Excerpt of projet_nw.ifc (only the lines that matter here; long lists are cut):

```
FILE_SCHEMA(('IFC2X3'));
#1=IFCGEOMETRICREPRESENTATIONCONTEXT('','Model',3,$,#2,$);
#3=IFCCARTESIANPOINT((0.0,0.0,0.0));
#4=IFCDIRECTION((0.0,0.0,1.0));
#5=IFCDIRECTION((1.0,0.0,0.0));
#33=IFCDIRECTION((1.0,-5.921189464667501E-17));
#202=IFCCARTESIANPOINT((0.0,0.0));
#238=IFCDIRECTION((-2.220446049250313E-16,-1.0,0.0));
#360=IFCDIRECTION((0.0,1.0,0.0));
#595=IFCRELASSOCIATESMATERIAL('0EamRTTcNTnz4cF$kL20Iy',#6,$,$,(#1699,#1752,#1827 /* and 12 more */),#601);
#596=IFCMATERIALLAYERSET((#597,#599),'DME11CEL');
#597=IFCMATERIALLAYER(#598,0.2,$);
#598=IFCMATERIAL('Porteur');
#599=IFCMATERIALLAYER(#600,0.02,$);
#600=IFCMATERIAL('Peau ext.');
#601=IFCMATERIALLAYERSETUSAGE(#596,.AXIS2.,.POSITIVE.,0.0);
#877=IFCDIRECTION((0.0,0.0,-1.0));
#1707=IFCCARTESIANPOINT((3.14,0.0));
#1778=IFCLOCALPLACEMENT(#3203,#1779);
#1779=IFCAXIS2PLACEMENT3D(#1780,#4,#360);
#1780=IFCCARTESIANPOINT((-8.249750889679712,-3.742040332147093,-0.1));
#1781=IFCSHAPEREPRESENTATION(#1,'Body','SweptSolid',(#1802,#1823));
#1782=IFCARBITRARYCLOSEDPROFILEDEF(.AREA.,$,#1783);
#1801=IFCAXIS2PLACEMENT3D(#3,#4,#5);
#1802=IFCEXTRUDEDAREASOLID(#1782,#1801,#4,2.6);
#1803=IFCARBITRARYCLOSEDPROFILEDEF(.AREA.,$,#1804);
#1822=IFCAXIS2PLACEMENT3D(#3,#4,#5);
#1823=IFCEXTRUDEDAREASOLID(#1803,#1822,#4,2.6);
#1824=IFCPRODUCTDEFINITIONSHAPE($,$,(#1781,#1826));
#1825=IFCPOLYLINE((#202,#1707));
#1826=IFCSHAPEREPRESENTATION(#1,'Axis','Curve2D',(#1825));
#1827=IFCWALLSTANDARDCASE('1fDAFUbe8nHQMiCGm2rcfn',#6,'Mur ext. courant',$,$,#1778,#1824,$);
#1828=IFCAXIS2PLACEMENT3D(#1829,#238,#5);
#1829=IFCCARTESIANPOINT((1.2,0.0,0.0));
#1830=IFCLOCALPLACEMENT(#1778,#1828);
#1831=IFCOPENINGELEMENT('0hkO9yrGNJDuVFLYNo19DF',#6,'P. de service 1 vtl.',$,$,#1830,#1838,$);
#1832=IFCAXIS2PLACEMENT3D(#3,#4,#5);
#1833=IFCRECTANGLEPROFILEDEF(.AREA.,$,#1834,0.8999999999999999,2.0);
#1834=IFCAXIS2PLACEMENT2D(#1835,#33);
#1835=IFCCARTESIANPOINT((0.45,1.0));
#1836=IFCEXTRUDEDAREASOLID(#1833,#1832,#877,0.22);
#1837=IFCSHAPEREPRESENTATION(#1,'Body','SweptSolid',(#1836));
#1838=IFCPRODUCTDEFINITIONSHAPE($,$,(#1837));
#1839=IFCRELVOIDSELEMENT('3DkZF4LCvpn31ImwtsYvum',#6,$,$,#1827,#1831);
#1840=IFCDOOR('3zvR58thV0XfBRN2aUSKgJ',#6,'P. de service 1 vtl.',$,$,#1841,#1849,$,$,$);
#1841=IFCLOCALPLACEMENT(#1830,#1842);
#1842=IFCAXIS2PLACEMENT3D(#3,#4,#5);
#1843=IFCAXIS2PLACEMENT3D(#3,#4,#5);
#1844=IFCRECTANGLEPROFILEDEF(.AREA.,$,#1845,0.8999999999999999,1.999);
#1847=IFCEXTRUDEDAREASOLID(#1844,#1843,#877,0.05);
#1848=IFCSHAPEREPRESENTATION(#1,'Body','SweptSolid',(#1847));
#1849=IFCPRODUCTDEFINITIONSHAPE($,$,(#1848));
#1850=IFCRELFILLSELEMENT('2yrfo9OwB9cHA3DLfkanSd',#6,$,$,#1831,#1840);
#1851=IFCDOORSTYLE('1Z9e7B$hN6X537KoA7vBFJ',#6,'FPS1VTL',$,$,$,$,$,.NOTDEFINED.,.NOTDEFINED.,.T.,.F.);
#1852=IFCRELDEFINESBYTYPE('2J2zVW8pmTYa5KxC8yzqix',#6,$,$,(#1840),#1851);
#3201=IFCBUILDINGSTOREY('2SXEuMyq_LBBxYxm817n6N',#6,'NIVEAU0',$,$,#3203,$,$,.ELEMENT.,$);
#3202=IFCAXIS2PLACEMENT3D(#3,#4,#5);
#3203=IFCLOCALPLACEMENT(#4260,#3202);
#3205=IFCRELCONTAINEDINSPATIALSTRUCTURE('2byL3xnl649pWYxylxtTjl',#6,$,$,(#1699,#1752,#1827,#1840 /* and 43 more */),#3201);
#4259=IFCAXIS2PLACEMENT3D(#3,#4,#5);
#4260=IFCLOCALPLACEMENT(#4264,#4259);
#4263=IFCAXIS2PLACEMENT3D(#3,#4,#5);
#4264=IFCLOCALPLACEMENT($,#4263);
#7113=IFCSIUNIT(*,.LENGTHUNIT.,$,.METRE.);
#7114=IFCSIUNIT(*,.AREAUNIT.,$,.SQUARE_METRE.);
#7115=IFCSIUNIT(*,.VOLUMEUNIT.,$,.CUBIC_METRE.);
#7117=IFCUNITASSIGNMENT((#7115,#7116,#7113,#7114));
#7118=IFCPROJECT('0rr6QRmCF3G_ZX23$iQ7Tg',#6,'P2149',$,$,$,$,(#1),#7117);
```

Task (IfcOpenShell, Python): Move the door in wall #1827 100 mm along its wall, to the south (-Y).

```python
import ifcopenshell
import ifcopenshell.api.geometry
import ifcopenshell.util.placement
import ifcopenshell.util.unit

model = ifcopenshell.open("projet_nw.ifc")
unit_scale = ifcopenshell.util.unit.calculate_unit_scale(model)

door = model.by_id(1840)
opening = door.FillsVoids[0].RelatingOpeningElement
wall = opening.VoidsElements[0].RelatingBuildingElement

wall_matrix = ifcopenshell.util.placement.get_local_placement(wall.ObjectPlacement)
shift = wall_matrix[:3, 0] * -0.1 / unit_scale
before = ifcopenshell.util.placement.get_local_placement(door.ObjectPlacement)[:3, 3].copy()

# The door is placed relative to its opening, so it follows when the opening moves.
matrix = ifcopenshell.util.placement.get_local_placement(opening.ObjectPlacement)
matrix[:3, 3] += shift
ifcopenshell.api.geometry.edit_object_placement(
    model, product=opening, matrix=matrix, is_si=False, should_transform_children=True
)

after = ifcopenshell.util.placement.get_local_placement(door.ObjectPlacement)[:3, 3]
print("door moved by", (after - before).round(3) + 0.0)

model.write("projet_nw_v2.ifc")
```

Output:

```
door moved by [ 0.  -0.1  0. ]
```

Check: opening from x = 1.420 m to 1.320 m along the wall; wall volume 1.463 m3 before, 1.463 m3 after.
